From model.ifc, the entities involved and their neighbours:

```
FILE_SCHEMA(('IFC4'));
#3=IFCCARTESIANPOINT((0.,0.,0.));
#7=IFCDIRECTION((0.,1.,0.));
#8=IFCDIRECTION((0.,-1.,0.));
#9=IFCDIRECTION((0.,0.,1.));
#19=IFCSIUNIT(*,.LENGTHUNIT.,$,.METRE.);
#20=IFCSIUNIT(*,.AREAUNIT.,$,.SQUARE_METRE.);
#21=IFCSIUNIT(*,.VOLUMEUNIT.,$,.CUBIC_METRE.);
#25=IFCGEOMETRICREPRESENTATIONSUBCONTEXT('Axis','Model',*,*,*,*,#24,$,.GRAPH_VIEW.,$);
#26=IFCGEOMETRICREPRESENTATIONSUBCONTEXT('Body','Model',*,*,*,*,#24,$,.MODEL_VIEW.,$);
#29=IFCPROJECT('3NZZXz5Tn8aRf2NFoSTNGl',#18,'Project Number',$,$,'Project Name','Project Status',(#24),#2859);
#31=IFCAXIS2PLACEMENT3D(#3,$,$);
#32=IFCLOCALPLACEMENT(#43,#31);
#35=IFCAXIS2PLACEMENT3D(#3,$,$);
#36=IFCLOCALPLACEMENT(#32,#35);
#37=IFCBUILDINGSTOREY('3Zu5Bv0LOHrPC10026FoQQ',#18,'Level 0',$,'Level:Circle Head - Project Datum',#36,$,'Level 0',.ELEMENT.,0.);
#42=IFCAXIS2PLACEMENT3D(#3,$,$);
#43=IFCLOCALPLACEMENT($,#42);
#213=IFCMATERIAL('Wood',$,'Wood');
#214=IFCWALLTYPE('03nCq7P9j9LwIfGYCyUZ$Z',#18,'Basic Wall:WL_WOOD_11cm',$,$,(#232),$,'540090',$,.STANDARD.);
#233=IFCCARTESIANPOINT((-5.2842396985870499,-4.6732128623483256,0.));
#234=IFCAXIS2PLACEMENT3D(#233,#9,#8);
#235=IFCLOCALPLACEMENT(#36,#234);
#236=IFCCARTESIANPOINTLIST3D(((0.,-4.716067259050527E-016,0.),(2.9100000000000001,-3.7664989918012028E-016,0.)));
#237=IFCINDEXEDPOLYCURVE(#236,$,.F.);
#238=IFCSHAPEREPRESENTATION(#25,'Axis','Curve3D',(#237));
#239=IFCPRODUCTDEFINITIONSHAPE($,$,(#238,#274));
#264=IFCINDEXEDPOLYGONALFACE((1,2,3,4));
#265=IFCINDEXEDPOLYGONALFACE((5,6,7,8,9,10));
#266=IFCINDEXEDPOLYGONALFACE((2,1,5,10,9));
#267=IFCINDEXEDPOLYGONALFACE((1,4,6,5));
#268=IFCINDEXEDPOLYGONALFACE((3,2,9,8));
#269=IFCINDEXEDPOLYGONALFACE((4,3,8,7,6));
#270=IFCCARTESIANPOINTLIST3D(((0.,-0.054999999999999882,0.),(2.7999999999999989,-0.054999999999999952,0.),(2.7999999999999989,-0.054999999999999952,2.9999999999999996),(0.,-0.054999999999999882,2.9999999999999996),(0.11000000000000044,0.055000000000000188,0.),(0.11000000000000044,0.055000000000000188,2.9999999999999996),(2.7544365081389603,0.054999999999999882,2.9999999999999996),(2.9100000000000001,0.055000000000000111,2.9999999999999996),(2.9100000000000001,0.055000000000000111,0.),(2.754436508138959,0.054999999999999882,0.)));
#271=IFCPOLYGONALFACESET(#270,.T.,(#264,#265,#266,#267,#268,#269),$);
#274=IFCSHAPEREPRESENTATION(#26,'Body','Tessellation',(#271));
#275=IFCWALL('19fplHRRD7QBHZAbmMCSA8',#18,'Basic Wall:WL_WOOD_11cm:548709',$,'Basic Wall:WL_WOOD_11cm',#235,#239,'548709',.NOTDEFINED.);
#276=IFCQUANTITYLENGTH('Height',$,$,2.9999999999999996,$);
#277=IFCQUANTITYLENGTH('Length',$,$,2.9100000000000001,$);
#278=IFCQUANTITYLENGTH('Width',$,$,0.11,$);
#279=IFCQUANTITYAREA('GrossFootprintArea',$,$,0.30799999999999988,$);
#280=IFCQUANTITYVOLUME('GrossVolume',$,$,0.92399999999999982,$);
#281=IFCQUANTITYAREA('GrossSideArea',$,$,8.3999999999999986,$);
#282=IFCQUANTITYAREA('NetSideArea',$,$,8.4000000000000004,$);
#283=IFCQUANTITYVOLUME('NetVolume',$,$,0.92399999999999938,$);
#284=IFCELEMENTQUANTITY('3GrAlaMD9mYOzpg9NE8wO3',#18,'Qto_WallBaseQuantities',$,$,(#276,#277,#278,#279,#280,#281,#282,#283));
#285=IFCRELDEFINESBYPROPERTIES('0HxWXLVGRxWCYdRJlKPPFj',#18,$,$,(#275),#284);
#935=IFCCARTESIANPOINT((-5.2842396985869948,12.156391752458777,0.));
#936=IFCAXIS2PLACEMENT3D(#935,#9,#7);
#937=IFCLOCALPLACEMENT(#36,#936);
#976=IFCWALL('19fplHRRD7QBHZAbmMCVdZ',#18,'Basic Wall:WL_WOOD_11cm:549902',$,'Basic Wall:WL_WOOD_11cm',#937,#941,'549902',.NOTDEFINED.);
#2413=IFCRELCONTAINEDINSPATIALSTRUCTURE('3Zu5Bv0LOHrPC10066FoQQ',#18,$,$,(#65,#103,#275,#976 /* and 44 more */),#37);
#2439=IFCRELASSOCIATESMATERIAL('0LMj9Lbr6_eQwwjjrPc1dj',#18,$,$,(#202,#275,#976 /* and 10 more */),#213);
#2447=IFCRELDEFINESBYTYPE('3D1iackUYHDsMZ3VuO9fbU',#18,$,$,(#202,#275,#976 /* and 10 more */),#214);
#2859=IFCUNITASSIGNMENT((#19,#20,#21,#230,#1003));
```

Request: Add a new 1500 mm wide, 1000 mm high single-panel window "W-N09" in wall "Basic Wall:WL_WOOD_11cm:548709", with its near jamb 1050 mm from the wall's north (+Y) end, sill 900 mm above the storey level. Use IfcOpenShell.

```python
import numpy as np
import ifcopenshell
import ifcopenshell.api.feature
import ifcopenshell.api.geometry
import ifcopenshell.api.pset
import ifcopenshell.api.root
import ifcopenshell.api.spatial
import ifcopenshell.geom
import ifcopenshell.util.element
import ifcopenshell.util.placement
import ifcopenshell.util.representation
import ifcopenshell.util.shape
import ifcopenshell.util.unit

model = ifcopenshell.open("model.ifc")
unit_scale = ifcopenshell.util.unit.calculate_unit_scale(model)
area_scale = ifcopenshell.util.unit.calculate_unit_scale(model, "AREAUNIT")
volume_scale = ifcopenshell.util.unit.calculate_unit_scale(model, "VOLUMEUNIT")
settings = ifcopenshell.geom.settings()


def volume(element):
    """Net volume in cubic metres, openings subtracted."""
    shape = ifcopenshell.geom.create_shape(settings, element)
    return ifcopenshell.util.shape.get_volume(shape.geometry)


wall = model.by_guid("19fplHRRD7QBHZAbmMCSA8")
storey = ifcopenshell.util.element.get_container(wall, ifc_class="IfcBuildingStorey")
context = ifcopenshell.util.representation.get_context(model, "Model", "Body", "MODEL_VIEW")
before = volume(wall)

width, height, from_end, sill = 1.5, 1, 1.05, 0.9  # metres

# The wall runs along its own X axis, and the end named is its -X end.
wall_shape = ifcopenshell.geom.create_shape(settings, wall)
x, y, z = ifcopenshell.util.shape.get_vertices(wall_shape.geometry).T
start = x.min() + from_end
face, thickness = float(y.min()), float(y.max() - y.min())
wall_matrix = ifcopenshell.util.placement.get_local_placement(wall.ObjectPlacement)
level = ifcopenshell.util.placement.get_local_placement(storey.ObjectPlacement)[2, 3]


def in_wall(x, y):
    """Placement at x, y metres in the wall's axes, at sill height."""
    matrix = wall_matrix.copy()
    matrix[:, 3] = wall_matrix @ np.array([x / unit_scale, y / unit_scale, 0.0, 1.0])
    matrix[2, 3] = level + sill / unit_scale
    return matrix


# Opening: a box that overshoots both wall faces by 50 mm.
opening = ifcopenshell.api.root.create_entity(model, ifc_class="IfcOpeningElement", predefined_type="OPENING")
box = ifcopenshell.api.geometry.add_wall_representation(
    model, context=context, length=width, height=height, thickness=thickness + 0.1
)
ifcopenshell.api.geometry.assign_representation(model, product=opening, representation=box)
ifcopenshell.api.geometry.edit_object_placement(model, product=opening, matrix=in_wall(start, face - 0.05), is_si=False)
ifcopenshell.api.feature.add_feature(model, feature=opening, element=wall)

window = ifcopenshell.api.root.create_entity(model, ifc_class="IfcWindow", name="W-N09", predefined_type="WINDOW")
window.OverallWidth, window.OverallHeight = width / unit_scale, height / unit_scale
window.PartitioningType = "SINGLE_PANEL"
body = ifcopenshell.api.geometry.add_window_representation(
    model,
    context=context,
    overall_width=window.OverallWidth,
    overall_height=window.OverallHeight,
    partition_type="SINGLE_PANEL",
)
ifcopenshell.api.geometry.assign_representation(model, product=window, representation=body)
ifcopenshell.api.spatial.assign_container(model, products=[window], relating_structure=storey)
ifcopenshell.api.feature.add_filling(model, opening=opening, element=window)

# Centre the window in the wall's thickness.
ifcopenshell.api.geometry.edit_object_placement(model, product=window, matrix=in_wall(start, face), is_si=False)
window_shape = ifcopenshell.geom.create_shape(settings, window)
depth = ifcopenshell.util.shape.get_vertices(window_shape.geometry)[:, 1]
offset = face + thickness / 2 - (depth.min() + depth.max()) / 2
ifcopenshell.api.geometry.edit_object_placement(model, product=window, matrix=in_wall(start, offset), is_si=False)

after = volume(wall)

# Update the wall's stored quantities.
qto = model.by_id(ifcopenshell.util.element.get_pset(wall, "Qto_WallBaseQuantities", should_inherit=False)["id"])
ifcopenshell.api.pset.edit_qto(model, qto=qto, properties={
    "NetSideArea": after / thickness / area_scale,
    "NetVolume": after / volume_scale,
})

print(f"wall volume {before:.3f} -> {after:.3f} m3")

model.write("model-out.ifc")
```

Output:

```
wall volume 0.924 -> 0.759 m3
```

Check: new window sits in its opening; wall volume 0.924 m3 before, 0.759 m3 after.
